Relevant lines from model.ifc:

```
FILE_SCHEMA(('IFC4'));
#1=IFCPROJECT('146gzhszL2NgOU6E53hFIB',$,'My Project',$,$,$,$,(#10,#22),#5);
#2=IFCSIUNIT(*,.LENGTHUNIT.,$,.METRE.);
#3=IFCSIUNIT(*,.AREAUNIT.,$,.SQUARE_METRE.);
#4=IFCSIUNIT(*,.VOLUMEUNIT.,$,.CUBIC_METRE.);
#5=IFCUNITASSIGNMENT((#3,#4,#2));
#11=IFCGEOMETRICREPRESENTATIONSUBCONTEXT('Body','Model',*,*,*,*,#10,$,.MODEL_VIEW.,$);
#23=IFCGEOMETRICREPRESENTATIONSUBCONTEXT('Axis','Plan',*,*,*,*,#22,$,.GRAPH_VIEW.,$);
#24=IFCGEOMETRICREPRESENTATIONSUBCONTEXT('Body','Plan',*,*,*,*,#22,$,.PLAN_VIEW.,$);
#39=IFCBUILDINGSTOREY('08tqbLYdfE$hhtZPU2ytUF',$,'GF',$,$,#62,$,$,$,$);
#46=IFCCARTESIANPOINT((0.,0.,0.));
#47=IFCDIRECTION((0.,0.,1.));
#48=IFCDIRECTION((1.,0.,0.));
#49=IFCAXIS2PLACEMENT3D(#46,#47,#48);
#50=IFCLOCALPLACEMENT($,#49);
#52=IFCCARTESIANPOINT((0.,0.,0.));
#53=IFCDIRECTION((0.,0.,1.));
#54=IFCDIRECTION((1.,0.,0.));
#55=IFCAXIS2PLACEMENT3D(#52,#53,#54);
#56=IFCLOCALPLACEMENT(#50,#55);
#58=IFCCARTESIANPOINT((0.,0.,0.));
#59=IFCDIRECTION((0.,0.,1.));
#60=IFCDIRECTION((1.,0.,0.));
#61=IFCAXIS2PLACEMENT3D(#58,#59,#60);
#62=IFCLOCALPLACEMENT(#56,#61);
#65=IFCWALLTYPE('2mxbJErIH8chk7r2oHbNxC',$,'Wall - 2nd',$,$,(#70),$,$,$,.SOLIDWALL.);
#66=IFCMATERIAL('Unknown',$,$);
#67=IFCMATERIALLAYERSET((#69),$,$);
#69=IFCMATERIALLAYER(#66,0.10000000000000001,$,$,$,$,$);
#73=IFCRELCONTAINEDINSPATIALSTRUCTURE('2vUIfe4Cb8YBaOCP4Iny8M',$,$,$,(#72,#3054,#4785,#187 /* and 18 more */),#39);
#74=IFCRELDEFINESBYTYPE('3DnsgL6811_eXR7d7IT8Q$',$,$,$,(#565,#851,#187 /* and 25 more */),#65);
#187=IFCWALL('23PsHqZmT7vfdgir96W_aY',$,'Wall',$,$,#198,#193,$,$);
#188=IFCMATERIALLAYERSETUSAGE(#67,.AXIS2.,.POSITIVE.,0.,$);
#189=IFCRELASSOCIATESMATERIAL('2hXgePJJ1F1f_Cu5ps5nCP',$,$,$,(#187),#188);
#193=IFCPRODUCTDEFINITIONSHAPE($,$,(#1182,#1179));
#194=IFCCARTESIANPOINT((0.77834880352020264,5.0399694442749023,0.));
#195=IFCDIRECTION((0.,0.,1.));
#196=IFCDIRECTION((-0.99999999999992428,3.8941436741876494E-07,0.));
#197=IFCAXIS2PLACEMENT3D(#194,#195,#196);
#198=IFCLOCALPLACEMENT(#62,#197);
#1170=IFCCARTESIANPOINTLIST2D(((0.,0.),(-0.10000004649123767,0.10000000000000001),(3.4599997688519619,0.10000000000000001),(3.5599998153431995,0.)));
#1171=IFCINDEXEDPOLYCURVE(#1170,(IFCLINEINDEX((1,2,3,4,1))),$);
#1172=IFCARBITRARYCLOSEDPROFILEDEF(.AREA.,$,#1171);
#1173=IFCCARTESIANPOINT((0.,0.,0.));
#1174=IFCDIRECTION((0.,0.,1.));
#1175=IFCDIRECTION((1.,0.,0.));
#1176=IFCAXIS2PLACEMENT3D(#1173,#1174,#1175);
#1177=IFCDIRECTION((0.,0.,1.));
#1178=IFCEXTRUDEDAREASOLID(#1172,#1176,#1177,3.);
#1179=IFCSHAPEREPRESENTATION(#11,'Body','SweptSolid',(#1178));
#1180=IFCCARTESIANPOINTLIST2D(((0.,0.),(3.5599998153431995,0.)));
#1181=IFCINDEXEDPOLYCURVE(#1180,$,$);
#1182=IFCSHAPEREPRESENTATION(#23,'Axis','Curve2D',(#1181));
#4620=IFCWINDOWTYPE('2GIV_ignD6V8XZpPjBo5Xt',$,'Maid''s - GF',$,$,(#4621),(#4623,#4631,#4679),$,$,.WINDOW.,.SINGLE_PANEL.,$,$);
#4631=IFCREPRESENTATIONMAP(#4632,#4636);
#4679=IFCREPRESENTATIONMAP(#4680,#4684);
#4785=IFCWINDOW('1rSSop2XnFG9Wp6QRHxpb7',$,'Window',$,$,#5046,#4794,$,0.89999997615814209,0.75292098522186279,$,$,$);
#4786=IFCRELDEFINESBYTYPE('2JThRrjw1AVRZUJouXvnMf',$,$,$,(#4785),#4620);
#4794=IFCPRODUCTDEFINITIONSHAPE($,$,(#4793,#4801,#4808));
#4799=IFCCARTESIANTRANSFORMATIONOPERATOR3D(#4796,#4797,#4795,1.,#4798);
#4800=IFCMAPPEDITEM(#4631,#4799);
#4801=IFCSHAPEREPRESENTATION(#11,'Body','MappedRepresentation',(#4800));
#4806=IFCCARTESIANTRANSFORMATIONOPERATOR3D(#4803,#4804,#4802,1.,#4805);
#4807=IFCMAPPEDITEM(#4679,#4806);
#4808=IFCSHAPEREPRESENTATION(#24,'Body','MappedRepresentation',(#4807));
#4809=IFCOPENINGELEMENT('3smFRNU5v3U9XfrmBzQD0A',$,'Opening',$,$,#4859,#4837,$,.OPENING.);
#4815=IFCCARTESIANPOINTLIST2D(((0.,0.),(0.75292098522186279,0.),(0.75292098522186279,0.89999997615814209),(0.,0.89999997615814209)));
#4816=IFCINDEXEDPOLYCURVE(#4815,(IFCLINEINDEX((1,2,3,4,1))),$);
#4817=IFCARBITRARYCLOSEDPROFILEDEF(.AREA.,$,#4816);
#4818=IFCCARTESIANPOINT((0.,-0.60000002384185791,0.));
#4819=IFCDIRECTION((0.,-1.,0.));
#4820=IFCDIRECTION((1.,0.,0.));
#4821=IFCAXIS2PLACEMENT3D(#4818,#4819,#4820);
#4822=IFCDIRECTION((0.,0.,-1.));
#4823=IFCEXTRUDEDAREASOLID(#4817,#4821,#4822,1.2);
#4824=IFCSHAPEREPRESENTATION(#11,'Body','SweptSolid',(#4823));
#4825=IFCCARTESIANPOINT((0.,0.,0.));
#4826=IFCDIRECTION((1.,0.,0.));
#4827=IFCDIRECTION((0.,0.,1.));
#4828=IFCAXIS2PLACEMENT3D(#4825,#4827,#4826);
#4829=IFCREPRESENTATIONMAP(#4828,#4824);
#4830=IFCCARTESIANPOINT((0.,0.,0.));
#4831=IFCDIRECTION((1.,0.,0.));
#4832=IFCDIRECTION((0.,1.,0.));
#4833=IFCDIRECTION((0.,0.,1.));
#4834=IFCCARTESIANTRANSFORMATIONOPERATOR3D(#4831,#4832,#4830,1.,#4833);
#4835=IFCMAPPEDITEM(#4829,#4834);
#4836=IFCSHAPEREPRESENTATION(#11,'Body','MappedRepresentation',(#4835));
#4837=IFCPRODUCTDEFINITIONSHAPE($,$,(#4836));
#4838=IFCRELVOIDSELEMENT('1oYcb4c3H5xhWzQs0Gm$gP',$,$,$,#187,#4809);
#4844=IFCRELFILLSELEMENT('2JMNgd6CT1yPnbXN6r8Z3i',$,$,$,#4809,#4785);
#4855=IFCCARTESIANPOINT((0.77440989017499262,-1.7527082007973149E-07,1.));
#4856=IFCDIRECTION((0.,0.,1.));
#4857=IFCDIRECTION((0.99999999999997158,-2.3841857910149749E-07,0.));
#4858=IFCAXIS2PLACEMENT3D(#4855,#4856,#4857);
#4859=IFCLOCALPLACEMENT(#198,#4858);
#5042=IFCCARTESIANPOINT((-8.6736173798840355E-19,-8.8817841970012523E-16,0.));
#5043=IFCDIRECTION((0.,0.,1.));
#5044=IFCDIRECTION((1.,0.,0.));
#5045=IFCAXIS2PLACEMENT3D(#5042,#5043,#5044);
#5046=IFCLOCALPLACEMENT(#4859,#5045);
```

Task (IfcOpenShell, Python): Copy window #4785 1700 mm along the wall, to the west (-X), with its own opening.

```python
import ifcopenshell
import ifcopenshell.api.feature
import ifcopenshell.api.geometry
import ifcopenshell.api.root
import ifcopenshell.geom
import ifcopenshell.util.element
import ifcopenshell.util.placement
import ifcopenshell.util.shape
import ifcopenshell.util.unit

model = ifcopenshell.open("model.ifc")
unit_scale = ifcopenshell.util.unit.calculate_unit_scale(model)
settings = ifcopenshell.geom.settings()


def volume(element):
    """Net volume in cubic metres, openings subtracted."""
    shape = ifcopenshell.geom.create_shape(settings, element)
    return ifcopenshell.util.shape.get_volume(shape.geometry)


window = model.by_guid("1rSSop2XnFG9Wp6QRHxpb7")
opening = window.FillsVoids[0].RelatingOpeningElement
wall = opening.VoidsElements[0].RelatingBuildingElement
before = volume(wall)
shift = ifcopenshell.util.placement.get_local_placement(wall.ObjectPlacement)[:3, 0] * 1.7 / unit_scale

# copy_class copies the void relationship, type, container and properties, but no geometry.
new_opening = ifcopenshell.api.root.copy_class(model, product=opening)
new_opening.Representation = ifcopenshell.util.element.copy_deep(
    model, opening.Representation, exclude=["IfcGeometricRepresentationContext", "IfcRepresentationMap"]
)
new_window = ifcopenshell.api.root.copy_class(model, product=window)
new_window.Representation = ifcopenshell.util.element.copy_deep(
    model, window.Representation, exclude=["IfcGeometricRepresentationContext", "IfcRepresentationMap"]
)
ifcopenshell.api.feature.add_filling(model, opening=new_opening, element=new_window)

for old, new in ((opening, new_opening), (window, new_window)):
    matrix = ifcopenshell.util.placement.get_local_placement(old.ObjectPlacement)
    matrix[:3, 3] += shift
    ifcopenshell.api.geometry.edit_object_placement(model, product=new, matrix=matrix, is_si=False)

after = volume(wall)

print(f"wall volume {before:.3f} -> {after:.3f} m3")

model.write("model_rev.ifc")
```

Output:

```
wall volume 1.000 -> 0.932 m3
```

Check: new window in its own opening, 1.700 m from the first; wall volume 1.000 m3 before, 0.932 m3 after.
